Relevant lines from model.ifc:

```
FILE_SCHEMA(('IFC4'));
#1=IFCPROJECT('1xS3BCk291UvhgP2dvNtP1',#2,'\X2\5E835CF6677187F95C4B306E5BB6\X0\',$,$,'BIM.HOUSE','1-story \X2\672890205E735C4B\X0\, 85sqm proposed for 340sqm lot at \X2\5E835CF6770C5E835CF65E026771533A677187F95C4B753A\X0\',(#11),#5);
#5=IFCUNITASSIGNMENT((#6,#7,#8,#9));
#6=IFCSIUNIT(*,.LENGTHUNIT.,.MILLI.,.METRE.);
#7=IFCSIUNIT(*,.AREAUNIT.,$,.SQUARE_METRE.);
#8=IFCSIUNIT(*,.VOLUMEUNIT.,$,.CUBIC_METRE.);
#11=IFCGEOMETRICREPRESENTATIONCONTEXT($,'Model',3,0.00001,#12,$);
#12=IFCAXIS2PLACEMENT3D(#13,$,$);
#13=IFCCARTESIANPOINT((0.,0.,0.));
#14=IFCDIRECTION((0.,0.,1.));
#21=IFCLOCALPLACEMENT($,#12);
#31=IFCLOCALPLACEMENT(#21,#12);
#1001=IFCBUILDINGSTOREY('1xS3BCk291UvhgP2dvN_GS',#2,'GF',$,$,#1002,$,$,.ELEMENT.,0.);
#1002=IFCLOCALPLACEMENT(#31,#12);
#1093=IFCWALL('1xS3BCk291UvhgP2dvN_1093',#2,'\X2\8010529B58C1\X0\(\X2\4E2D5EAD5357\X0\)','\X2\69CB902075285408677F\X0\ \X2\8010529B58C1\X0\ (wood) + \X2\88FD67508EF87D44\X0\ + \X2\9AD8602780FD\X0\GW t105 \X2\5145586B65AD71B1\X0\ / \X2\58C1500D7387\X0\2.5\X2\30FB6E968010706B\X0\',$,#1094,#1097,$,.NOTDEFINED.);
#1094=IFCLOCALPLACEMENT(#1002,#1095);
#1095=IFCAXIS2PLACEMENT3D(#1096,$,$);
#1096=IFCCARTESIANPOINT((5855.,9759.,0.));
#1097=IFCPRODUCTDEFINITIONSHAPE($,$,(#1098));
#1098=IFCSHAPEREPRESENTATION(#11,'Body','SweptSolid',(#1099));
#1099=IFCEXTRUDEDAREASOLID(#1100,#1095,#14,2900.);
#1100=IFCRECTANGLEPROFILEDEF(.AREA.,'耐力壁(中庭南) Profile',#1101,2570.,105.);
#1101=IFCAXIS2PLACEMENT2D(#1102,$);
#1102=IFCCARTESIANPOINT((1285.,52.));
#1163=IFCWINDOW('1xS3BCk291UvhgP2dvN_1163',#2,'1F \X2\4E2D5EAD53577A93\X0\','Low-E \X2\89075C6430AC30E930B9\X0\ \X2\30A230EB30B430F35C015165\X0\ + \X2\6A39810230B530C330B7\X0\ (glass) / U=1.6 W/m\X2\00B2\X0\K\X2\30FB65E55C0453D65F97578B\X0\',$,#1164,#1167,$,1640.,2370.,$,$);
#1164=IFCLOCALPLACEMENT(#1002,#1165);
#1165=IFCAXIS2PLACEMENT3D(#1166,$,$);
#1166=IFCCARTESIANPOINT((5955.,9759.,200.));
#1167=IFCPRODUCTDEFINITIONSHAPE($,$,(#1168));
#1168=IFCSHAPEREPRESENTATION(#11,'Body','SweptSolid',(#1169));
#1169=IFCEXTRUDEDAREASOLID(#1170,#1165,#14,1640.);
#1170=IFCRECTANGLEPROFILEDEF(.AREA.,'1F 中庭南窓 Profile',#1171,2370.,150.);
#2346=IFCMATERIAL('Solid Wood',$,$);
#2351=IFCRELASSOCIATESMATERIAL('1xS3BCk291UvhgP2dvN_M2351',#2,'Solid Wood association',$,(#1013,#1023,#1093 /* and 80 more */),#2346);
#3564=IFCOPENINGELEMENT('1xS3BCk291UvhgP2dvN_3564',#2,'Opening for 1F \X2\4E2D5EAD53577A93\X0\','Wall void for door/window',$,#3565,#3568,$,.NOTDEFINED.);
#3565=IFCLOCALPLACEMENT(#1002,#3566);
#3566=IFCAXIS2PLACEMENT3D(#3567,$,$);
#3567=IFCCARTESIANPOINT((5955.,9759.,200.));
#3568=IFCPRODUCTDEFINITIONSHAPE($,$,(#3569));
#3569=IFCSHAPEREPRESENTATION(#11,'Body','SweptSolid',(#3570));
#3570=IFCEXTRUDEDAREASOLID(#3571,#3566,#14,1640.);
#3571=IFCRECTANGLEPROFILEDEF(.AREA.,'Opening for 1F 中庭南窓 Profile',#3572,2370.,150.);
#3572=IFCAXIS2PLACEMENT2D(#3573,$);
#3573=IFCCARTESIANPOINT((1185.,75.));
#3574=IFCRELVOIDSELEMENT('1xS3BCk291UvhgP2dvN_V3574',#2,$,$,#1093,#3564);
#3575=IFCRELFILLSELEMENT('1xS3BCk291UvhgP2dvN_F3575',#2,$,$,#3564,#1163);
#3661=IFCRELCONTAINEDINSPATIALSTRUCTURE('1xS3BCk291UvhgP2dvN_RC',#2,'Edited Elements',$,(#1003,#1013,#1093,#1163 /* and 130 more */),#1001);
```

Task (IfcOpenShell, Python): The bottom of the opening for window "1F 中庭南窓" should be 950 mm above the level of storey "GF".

```python
import numpy as np
import ifcopenshell
import ifcopenshell.api.geometry
import ifcopenshell.geom
import ifcopenshell.util.element
import ifcopenshell.util.placement
import ifcopenshell.util.shape
import ifcopenshell.util.unit

model = ifcopenshell.open("model.ifc")
unit_scale = ifcopenshell.util.unit.calculate_unit_scale(model)

window = model.by_id(1163)
opening = window.FillsVoids[0].RelatingOpeningElement
storey = ifcopenshell.util.element.get_container(window, ifc_class="IfcBuildingStorey")
level = ifcopenshell.util.placement.get_local_placement(storey.ObjectPlacement)[2, 3]

# The opening's origin need not be at the sill, so measure its lowest point.
shape = ifcopenshell.geom.create_shape(ifcopenshell.geom.settings(), opening)
bottom = ifcopenshell.util.shape.get_shape_bottom_elevation(shape, shape.geometry) / unit_scale
dz = level + 0.95 / unit_scale - bottom

shift = np.array([0.0, 0.0, dz])
# The window is not placed relative to its opening, so move both.
for product in (opening, window):
    matrix = ifcopenshell.util.placement.get_local_placement(product.ObjectPlacement)
    matrix[:3, 3] += shift
    ifcopenshell.api.geometry.edit_object_placement(model, product=product, matrix=matrix, is_si=False)

print(f"moved by {dz * unit_scale:+.3f} m")

model.write("model-out.ifc")
```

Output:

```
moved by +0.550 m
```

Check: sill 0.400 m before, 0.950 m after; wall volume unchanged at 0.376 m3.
